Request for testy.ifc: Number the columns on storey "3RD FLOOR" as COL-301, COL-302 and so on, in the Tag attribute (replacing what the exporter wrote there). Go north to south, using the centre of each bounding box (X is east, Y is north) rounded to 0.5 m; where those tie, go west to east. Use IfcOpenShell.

First a look at what the model holds.

```python
import ifcopenshell
import ifcopenshell.util.element
import ifcopenshell.util.placement

model = ifcopenshell.open("testy.ifc")
print(model.schema)
storey = next(s for s in model.by_type("IfcBuildingStorey") if s.Name == "3RD FLOOR")
columns = [e for e in ifcopenshell.util.element.get_decomposition(storey) if e.is_a("IfcColumn")]
for e in sorted(columns, key=lambda e: e.id()):
    origin = ifcopenshell.util.placement.get_local_placement(e.ObjectPlacement)[:3, 3]
    print(e.id(), e.Tag, e.Name, origin.round(2) + 0.0, sep=" | ")
```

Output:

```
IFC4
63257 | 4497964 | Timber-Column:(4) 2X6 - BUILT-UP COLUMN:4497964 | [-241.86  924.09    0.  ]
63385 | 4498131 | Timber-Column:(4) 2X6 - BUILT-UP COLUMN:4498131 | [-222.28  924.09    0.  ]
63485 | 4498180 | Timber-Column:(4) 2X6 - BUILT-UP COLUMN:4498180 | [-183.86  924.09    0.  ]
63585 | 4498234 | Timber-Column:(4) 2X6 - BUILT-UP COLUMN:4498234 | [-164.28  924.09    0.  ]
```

```python
import ifcopenshell
import ifcopenshell.geom
import ifcopenshell.util.element
import ifcopenshell.util.shape

model = ifcopenshell.open("testy.ifc")
settings = ifcopenshell.geom.settings()
settings.set("use-world-coords", True)


def centre(element):
    shape = ifcopenshell.geom.create_shape(settings, element)
    return ifcopenshell.util.shape.get_bbox_centroid(shape.geometry)


storey = next(s for s in model.by_type("IfcBuildingStorey") if s.Name == "3RD FLOOR")
columns = [e for e in ifcopenshell.util.element.get_decomposition(storey) if e.is_a("IfcColumn")]

# Insertion points can sit at a corner or the storey origin, so sort by the geometry (in metres).
centres = {e: centre(e) for e in columns}
columns.sort(key=lambda e: (-round(centres[e][1] / 0.5), centres[e][0]))

for i, e in enumerate(columns, start=1):
    number = f"COL-3{i:02d}"
    e.Tag = number
    print(e.id(), number)

model.write("testy_v2.ifc")
```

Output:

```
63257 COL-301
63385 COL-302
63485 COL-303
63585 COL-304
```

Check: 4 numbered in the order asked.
